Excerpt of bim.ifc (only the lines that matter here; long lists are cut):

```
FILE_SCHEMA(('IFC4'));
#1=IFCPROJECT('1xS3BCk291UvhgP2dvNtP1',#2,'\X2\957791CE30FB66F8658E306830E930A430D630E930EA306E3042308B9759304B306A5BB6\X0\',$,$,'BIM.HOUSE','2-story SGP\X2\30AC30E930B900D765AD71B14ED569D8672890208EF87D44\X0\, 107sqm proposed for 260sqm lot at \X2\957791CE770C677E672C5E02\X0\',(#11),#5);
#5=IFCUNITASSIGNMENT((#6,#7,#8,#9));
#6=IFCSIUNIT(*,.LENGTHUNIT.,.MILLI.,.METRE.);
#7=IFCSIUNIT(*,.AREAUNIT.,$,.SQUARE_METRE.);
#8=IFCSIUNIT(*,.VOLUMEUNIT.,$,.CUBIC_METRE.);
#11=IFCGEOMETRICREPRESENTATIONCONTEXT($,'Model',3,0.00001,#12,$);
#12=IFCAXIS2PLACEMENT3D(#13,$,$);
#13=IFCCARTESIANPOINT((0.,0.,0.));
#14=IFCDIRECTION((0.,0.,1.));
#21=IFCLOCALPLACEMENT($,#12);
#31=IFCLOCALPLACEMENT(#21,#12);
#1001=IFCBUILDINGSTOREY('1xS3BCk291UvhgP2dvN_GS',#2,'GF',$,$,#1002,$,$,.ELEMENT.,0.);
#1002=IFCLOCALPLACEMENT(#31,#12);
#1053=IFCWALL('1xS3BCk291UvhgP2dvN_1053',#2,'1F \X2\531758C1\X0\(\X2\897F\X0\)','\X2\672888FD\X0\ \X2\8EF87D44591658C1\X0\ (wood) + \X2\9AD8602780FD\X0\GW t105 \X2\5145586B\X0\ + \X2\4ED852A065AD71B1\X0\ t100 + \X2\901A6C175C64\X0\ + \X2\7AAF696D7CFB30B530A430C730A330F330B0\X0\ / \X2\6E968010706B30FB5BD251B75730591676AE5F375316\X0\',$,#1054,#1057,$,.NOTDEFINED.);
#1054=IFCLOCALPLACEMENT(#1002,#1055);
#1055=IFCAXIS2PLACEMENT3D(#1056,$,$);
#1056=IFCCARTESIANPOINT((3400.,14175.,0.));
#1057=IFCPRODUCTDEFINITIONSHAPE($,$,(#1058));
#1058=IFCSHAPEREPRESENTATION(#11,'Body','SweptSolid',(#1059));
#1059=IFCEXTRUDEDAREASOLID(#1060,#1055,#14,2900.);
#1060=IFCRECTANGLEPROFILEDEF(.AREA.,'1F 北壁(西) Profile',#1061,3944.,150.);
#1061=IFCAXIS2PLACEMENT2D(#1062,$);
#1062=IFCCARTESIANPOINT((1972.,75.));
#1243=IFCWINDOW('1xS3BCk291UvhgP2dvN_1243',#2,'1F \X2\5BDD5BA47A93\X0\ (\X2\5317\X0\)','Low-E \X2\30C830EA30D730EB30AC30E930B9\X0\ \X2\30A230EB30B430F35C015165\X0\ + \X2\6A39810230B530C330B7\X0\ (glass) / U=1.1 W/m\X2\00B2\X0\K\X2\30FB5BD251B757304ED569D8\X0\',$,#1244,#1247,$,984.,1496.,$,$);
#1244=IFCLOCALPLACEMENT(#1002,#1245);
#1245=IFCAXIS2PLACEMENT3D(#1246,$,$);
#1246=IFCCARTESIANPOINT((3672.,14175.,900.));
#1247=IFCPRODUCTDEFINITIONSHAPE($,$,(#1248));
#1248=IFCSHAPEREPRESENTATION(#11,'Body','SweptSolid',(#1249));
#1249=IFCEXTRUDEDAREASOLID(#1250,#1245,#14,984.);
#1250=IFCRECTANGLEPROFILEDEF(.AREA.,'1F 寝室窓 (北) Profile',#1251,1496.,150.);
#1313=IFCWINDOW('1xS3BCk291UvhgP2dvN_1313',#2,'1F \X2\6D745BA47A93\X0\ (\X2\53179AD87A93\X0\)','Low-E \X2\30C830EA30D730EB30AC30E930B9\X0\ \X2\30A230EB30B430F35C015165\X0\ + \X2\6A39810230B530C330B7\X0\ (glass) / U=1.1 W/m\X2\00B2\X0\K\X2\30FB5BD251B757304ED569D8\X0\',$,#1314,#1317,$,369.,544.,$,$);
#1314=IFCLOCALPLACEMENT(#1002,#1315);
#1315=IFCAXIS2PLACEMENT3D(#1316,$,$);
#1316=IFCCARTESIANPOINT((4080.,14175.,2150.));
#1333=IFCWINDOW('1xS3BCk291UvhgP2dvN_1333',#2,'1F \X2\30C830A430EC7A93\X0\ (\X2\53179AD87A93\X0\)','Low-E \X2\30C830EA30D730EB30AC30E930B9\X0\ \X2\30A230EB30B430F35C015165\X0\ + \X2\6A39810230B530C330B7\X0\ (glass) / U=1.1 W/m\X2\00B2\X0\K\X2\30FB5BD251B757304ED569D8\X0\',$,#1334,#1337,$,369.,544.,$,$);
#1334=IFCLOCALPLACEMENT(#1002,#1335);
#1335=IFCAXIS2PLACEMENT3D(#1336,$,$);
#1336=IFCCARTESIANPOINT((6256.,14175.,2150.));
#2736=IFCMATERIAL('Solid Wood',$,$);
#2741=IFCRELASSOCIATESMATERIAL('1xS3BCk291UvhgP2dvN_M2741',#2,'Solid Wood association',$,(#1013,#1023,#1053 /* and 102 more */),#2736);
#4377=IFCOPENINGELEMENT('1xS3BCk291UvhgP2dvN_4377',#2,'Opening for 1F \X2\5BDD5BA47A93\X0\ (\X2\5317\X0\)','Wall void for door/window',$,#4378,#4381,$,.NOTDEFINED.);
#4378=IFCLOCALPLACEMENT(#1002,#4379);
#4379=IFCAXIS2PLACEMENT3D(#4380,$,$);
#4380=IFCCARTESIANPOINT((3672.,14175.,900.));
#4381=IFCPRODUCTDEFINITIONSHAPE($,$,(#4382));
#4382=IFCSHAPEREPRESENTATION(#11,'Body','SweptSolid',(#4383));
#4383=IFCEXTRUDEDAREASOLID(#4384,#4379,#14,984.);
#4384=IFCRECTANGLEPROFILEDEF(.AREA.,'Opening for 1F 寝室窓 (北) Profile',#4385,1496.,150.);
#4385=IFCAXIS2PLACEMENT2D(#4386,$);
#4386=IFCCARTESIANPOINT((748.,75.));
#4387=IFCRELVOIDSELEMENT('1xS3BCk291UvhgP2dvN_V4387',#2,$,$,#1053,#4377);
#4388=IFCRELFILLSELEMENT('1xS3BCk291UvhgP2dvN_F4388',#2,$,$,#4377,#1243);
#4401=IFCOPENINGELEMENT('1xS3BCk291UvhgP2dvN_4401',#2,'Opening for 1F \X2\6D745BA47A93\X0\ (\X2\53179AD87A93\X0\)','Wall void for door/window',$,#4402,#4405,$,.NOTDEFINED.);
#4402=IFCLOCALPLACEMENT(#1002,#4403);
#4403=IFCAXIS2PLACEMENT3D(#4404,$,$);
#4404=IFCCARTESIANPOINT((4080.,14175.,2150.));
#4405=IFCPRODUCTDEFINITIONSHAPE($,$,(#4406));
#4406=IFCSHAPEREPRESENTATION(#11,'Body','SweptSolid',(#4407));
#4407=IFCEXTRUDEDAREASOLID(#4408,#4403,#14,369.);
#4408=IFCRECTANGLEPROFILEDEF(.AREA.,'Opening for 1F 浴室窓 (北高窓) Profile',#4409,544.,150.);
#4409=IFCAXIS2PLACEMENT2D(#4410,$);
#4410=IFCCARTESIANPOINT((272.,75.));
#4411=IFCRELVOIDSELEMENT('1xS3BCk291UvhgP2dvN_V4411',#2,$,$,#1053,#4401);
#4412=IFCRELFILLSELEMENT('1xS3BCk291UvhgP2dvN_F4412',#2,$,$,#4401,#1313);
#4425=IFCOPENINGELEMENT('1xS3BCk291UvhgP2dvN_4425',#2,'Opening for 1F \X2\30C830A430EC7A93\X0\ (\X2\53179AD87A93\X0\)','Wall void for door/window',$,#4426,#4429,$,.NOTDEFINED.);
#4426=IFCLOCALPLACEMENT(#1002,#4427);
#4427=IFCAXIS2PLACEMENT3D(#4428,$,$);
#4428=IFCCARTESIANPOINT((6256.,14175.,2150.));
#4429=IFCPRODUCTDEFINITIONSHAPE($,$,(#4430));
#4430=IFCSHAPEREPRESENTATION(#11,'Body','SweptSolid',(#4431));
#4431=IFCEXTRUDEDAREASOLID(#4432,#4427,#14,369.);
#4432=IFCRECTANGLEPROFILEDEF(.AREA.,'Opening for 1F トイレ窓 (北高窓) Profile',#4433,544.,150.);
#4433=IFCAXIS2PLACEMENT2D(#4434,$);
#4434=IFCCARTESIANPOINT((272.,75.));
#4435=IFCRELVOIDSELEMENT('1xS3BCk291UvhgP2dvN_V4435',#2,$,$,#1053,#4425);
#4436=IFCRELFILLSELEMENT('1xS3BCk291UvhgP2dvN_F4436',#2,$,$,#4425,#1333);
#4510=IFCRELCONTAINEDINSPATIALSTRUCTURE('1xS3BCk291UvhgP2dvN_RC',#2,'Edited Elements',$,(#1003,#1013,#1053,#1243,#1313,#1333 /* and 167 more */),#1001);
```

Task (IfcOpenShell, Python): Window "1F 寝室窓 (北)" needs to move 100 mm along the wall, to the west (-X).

```python
import ifcopenshell
import ifcopenshell.api.geometry
import ifcopenshell.util.placement
import ifcopenshell.util.unit

model = ifcopenshell.open("bim.ifc")
unit_scale = ifcopenshell.util.unit.calculate_unit_scale(model)

window = model.by_id(1243)
opening = window.FillsVoids[0].RelatingOpeningElement
wall = opening.VoidsElements[0].RelatingBuildingElement

wall_matrix = ifcopenshell.util.placement.get_local_placement(wall.ObjectPlacement)
shift = wall_matrix[:3, 0] * -0.1 / unit_scale
before = ifcopenshell.util.placement.get_local_placement(window.ObjectPlacement)[:3, 3].copy()

# The window is not placed relative to its opening, so move both.
for product in (opening, window):
    matrix = ifcopenshell.util.placement.get_local_placement(product.ObjectPlacement)
    matrix[:3, 3] += shift
    ifcopenshell.api.geometry.edit_object_placement(model, product=product, matrix=matrix, is_si=False)

after = ifcopenshell.util.placement.get_local_placement(window.ObjectPlacement)[:3, 3]
print("window moved by", (after - before).round(3) + 0.0)

model.write("bim_updated.ifc")
```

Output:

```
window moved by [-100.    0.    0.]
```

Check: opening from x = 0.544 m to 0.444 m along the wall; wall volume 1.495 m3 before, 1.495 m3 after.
